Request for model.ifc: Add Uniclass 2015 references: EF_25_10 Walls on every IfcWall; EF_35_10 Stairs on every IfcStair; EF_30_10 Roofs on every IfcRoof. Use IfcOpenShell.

First a look at what the model holds.

```python
import ifcopenshell

model = ifcopenshell.open("model.ifc")
print(model.schema)
print("classifications:", [c.Name for c in model.by_type("IfcClassification")])
for ifc_class in ("IfcDoor", "IfcRoof", "IfcStair", "IfcWall", "IfcWindow"):
    print(ifc_class, len(model.by_type(ifc_class)))
```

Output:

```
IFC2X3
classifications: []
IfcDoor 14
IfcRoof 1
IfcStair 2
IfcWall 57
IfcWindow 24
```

```python
import ifcopenshell
import ifcopenshell.api.classification

model = ifcopenshell.open("model.ifc")

# IFC2X3 requires Source and Edition and has no link from the project to the system.
system = model.create_entity("IfcClassification", Source="NBS", Edition="2015", Name="Uniclass 2015")

codes = {
    "IfcWall": ("EF_25_10", "Walls"),
    "IfcStair": ("EF_35_10", "Stairs"),
    "IfcRoof": ("EF_30_10", "Roofs"),
}
for ifc_class, (code, name) in codes.items():
    products = model.by_type(ifc_class)
    ifcopenshell.api.classification.add_reference(
        model, products=products, classification=system, identification=code, name=name
    )
    print(code, len(products))

model.write("model_edited.ifc")
```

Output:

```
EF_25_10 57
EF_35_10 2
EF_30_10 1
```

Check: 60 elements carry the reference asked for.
